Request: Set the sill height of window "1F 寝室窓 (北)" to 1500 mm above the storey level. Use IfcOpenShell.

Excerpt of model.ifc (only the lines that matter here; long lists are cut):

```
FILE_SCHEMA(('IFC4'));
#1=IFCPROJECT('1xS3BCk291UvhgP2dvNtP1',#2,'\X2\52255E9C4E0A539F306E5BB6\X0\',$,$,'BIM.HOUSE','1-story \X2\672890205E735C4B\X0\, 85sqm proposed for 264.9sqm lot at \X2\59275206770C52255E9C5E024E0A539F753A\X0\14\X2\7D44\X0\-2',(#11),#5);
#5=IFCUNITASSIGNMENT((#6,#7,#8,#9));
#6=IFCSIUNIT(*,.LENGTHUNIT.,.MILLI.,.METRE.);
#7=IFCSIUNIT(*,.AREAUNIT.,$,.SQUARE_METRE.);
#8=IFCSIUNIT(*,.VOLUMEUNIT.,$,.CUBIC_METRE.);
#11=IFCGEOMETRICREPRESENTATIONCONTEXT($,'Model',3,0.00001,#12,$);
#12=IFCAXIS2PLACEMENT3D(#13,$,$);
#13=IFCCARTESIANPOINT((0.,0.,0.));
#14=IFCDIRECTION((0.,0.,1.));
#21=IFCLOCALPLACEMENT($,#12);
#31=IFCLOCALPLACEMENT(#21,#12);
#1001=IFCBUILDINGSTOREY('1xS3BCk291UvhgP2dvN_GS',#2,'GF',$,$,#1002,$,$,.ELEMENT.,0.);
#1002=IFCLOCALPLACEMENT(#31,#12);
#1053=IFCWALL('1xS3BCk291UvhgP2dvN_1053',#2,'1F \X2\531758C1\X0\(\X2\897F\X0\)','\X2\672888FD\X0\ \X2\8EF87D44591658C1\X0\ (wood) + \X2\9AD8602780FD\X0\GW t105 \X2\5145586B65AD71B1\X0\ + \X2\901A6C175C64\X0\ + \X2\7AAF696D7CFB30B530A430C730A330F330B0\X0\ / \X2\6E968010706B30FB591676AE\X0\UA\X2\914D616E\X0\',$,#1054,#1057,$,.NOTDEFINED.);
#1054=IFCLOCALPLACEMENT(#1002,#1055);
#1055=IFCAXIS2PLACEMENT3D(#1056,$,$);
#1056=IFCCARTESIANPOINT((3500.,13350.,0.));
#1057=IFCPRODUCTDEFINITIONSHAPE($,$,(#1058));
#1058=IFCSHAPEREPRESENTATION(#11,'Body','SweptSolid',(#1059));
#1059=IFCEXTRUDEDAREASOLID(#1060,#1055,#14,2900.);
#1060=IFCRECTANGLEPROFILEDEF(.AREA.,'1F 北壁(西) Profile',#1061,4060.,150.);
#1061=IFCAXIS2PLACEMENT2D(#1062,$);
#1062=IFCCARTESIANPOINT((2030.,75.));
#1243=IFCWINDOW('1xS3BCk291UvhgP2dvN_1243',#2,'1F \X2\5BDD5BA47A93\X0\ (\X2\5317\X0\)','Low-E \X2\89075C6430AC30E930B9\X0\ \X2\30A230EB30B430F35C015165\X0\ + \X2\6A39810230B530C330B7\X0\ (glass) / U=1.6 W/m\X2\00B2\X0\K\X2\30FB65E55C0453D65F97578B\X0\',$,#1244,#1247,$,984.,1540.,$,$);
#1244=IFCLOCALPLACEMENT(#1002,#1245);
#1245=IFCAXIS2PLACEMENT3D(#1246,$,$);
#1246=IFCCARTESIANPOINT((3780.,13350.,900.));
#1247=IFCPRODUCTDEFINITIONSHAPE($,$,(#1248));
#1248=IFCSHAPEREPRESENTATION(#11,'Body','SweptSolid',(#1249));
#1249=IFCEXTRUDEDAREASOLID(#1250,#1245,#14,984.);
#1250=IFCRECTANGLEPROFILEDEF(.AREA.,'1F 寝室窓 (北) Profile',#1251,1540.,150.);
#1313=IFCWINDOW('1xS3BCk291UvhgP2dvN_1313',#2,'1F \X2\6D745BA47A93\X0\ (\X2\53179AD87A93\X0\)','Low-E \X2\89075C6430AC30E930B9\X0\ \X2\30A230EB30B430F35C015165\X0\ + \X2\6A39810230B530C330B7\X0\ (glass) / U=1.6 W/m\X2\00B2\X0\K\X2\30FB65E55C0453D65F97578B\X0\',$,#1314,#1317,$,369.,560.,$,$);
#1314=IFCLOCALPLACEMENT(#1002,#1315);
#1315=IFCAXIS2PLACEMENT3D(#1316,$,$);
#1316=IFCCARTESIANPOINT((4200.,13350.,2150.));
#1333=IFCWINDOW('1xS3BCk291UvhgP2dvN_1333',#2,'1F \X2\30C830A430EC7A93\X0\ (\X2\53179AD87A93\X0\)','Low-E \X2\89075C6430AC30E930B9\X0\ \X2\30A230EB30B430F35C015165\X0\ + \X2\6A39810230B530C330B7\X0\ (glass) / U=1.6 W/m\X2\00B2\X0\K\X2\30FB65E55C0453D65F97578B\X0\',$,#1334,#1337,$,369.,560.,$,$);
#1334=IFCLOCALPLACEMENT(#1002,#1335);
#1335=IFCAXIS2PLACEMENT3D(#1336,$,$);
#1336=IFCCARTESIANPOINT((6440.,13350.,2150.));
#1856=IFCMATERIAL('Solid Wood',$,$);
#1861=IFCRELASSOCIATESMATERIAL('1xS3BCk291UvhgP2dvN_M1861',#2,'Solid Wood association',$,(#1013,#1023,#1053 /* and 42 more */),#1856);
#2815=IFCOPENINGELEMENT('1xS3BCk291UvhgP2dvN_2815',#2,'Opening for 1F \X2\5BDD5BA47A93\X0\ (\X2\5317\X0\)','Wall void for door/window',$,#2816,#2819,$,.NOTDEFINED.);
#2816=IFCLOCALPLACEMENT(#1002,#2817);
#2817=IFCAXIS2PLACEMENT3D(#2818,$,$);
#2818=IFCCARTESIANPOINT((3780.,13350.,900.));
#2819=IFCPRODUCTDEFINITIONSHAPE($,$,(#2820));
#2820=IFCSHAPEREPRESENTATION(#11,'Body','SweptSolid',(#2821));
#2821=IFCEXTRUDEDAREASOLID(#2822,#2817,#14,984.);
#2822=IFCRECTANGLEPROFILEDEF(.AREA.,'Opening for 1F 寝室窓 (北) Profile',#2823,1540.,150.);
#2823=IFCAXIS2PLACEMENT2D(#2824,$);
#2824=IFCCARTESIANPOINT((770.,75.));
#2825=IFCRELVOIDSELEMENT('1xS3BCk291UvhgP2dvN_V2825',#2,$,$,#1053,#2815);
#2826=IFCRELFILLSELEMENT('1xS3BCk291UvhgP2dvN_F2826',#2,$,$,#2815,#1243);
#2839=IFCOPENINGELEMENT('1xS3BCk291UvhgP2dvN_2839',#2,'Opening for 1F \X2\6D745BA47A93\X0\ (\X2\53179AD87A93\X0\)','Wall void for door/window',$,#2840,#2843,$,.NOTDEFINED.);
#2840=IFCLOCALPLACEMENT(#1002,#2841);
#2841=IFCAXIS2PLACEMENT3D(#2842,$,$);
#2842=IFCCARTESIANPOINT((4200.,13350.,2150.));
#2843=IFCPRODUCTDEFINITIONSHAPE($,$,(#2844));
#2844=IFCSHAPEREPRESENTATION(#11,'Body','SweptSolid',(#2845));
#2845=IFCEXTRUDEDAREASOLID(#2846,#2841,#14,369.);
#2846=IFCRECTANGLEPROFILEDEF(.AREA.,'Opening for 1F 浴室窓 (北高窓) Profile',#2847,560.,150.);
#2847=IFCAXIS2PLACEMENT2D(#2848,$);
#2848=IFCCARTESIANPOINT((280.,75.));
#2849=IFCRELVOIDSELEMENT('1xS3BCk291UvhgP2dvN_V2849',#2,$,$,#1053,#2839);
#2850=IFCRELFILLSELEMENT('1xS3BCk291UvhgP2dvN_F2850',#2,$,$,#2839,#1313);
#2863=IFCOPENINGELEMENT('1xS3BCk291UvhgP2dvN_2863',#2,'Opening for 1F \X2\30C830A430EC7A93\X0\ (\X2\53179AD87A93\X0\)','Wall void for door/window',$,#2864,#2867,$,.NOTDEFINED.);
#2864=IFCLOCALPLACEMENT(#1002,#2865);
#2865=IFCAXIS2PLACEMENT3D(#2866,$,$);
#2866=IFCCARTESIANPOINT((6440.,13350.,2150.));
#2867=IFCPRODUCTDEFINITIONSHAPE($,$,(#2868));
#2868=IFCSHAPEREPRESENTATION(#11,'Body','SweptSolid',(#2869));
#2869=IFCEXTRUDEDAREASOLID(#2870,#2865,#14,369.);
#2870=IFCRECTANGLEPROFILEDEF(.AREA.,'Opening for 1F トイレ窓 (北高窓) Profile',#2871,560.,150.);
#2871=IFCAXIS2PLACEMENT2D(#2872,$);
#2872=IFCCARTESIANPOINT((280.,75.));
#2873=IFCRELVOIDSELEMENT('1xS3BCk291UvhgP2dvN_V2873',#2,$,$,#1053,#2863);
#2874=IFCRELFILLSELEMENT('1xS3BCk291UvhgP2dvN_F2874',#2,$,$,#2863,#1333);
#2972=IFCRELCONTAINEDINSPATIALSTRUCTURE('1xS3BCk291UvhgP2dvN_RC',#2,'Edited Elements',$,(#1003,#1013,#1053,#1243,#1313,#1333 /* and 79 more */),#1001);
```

```python
import numpy as np
import ifcopenshell
import ifcopenshell.api.geometry
import ifcopenshell.geom
import ifcopenshell.util.element
import ifcopenshell.util.placement
import ifcopenshell.util.shape
import ifcopenshell.util.unit

model = ifcopenshell.open("model.ifc")
unit_scale = ifcopenshell.util.unit.calculate_unit_scale(model)

window = model.by_guid("1xS3BCk291UvhgP2dvN_1243")
opening = window.FillsVoids[0].RelatingOpeningElement
storey = ifcopenshell.util.element.get_container(window, ifc_class="IfcBuildingStorey")
level = ifcopenshell.util.placement.get_local_placement(storey.ObjectPlacement)[2, 3]

# The opening's origin need not be at the sill, so measure its lowest point.
shape = ifcopenshell.geom.create_shape(ifcopenshell.geom.settings(), opening)
bottom = ifcopenshell.util.shape.get_shape_bottom_elevation(shape, shape.geometry) / unit_scale
dz = level + 1500.0 - bottom

shift = np.array([0.0, 0.0, dz])
# The window is not placed relative to its opening, so move both.
for product in (opening, window):
    matrix = ifcopenshell.util.placement.get_local_placement(product.ObjectPlacement)
    matrix[:3, 3] += shift
    ifcopenshell.api.geometry.edit_object_placement(model, product=product, matrix=matrix, is_si=False)

print(f"moved by {dz * unit_scale:+.3f} m")

model.write("model_updated.ifc")
```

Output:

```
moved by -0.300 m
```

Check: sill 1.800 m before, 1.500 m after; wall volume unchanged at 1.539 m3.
